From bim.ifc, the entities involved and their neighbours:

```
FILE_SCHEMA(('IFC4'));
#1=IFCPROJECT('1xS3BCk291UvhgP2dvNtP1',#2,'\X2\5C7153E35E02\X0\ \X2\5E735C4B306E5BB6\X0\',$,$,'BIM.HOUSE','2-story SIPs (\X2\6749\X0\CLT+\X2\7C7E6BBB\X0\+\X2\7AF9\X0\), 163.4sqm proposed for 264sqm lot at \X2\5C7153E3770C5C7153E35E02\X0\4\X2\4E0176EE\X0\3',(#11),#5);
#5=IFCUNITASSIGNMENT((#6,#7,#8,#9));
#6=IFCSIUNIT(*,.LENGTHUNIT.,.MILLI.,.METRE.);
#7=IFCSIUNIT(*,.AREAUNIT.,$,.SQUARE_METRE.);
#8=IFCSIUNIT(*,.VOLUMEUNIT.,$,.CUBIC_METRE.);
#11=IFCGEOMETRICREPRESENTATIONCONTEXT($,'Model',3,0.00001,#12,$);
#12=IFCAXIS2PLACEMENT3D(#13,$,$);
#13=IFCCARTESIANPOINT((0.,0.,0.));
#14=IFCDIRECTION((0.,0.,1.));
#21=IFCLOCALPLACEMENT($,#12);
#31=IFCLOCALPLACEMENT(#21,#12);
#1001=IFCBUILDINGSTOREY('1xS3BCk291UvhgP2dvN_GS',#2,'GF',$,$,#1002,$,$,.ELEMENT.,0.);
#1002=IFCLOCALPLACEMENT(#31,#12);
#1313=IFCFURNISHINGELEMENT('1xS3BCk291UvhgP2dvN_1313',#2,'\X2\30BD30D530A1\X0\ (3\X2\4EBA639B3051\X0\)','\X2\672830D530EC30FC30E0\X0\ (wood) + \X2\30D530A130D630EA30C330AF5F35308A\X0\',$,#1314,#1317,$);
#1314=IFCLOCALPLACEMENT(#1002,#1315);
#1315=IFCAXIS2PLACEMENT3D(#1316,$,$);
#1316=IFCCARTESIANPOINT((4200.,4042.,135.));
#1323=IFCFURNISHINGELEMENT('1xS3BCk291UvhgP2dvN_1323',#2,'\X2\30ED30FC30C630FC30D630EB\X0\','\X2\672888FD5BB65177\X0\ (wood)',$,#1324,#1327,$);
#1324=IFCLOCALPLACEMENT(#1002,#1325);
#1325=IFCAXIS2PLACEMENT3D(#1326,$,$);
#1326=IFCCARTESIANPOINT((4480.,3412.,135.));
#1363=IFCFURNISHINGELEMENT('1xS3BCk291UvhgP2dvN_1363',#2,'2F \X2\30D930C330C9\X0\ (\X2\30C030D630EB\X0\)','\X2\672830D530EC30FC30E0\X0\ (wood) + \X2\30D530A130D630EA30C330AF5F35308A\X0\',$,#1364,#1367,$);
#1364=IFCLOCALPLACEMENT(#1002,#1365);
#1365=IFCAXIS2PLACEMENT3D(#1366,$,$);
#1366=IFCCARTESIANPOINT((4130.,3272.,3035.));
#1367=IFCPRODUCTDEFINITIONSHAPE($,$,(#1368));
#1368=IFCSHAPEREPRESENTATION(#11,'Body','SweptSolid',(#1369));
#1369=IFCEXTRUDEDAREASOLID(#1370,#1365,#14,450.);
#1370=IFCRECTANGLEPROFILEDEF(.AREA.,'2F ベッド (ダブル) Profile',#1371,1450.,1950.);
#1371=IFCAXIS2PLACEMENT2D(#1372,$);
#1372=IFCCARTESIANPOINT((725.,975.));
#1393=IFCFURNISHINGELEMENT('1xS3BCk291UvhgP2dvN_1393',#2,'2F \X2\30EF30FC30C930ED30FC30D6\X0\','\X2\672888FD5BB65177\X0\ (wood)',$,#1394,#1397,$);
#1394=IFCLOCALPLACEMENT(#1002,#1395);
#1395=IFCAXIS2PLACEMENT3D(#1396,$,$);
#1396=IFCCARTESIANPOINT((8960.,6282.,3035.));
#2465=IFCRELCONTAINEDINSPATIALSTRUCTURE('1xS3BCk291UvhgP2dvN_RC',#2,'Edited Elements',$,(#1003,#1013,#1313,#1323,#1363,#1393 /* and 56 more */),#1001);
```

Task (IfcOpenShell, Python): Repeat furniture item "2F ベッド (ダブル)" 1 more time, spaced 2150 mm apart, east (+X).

```python
import numpy as np
import ifcopenshell
import ifcopenshell.api.geometry
import ifcopenshell.api.root
import ifcopenshell.util.element
import ifcopenshell.util.placement

model = ifcopenshell.open("bim.ifc")


def reuse_history(source, copy):
    """copy_class also copies each property set's owner history, people and application; keep the originals."""
    for rel in copy.IsDefinedBy:
        if rel.is_a("IfcRelDefinesByProperties") and (history := rel.RelatingPropertyDefinition.OwnerHistory):
            rel.RelatingPropertyDefinition.OwnerHistory = source.OwnerHistory
            ifcopenshell.util.element.remove_deep2(model, history)


source = model.by_guid("1xS3BCk291UvhgP2dvN_1363")
base = ifcopenshell.util.placement.get_local_placement(source.ObjectPlacement)
step = np.array([1.0, 0.0, 0.0]) * 2150.0

for i in range(1, 2):
    copy = ifcopenshell.api.root.copy_class(model, product=source)
    copy.Representation = ifcopenshell.util.element.copy_deep(
        model, source.Representation, exclude=["IfcGeometricRepresentationContext", "IfcRepresentationMap"]
    )
    reuse_history(source, copy)
    matrix = base.copy()
    matrix[:3, 3] += i * step
    print("added at", matrix[:3, 3].round(3) + 0.0)
    ifcopenshell.api.geometry.edit_object_placement(model, product=copy, matrix=matrix, is_si=False)

model.write("bim_edited.ifc")
```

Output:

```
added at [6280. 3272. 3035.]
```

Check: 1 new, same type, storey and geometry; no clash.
